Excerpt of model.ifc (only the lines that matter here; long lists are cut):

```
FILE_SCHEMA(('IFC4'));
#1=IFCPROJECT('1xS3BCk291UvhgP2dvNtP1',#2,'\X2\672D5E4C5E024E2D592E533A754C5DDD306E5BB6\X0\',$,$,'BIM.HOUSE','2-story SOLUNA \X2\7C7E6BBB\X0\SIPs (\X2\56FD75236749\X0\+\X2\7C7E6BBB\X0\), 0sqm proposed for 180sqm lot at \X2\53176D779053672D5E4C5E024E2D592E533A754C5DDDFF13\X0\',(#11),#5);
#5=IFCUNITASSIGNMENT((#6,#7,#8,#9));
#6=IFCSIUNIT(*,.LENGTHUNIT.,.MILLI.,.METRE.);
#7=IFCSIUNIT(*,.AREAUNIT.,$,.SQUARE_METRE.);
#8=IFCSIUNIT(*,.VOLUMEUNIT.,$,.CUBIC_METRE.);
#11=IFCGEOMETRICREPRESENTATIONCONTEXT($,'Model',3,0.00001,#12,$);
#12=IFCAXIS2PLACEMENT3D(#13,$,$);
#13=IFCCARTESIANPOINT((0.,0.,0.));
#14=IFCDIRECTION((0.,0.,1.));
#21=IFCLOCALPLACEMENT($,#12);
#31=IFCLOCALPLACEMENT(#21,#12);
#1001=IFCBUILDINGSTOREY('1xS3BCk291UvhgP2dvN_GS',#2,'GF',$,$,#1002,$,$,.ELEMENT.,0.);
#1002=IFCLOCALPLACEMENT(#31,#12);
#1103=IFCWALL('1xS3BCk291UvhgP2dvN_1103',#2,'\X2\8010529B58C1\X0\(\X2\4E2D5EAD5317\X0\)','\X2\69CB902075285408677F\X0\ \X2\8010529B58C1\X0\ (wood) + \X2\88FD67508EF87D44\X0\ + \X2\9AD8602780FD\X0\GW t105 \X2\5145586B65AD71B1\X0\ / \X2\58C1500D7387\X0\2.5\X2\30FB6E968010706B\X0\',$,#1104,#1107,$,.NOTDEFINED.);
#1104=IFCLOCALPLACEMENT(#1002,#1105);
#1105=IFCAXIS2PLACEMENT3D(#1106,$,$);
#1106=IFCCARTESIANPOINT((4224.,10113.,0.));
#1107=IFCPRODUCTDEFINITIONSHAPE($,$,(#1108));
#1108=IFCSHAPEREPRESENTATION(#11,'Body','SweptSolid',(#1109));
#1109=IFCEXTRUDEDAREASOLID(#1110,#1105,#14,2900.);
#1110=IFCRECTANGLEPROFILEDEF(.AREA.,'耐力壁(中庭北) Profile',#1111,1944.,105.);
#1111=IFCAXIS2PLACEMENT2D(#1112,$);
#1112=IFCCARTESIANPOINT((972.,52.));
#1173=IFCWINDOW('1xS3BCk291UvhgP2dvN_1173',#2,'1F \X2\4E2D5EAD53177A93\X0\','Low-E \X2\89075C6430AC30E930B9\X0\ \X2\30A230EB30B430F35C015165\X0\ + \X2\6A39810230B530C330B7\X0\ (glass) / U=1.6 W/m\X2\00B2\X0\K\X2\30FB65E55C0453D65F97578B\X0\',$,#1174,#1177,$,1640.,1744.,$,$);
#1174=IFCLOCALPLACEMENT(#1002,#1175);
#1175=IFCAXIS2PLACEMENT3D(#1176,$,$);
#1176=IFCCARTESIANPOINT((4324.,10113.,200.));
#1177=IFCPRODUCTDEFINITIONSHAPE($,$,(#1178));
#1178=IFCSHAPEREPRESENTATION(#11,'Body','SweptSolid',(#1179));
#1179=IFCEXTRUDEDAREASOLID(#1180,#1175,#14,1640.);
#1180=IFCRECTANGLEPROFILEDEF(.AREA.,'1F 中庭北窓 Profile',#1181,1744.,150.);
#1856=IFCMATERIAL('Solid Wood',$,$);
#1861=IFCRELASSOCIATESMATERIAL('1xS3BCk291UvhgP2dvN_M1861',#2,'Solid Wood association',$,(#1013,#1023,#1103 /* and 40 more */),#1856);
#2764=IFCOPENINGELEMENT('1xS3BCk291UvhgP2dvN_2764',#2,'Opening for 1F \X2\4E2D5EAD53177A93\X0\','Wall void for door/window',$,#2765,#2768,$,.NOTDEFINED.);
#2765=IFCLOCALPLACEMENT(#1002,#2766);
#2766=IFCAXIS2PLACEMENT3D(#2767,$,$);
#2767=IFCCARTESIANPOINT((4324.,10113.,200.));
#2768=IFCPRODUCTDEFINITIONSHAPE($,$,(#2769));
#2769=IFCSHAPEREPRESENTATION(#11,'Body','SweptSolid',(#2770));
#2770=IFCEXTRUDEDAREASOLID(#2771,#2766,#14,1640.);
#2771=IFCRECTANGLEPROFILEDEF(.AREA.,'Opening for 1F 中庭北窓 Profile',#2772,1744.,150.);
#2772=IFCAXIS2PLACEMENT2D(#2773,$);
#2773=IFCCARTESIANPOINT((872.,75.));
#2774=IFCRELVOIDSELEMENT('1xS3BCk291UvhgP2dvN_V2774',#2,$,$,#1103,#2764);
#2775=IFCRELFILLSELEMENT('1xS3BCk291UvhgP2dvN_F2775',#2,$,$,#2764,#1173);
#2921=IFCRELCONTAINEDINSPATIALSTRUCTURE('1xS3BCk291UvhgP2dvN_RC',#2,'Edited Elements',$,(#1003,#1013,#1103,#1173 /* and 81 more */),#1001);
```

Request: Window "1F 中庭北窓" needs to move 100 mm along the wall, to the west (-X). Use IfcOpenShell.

```python
import ifcopenshell
import ifcopenshell.api.geometry
import ifcopenshell.util.placement

model = ifcopenshell.open("model.ifc")

window = model.by_id(1173)
opening = window.FillsVoids[0].RelatingOpeningElement
wall = opening.VoidsElements[0].RelatingBuildingElement

wall_matrix = ifcopenshell.util.placement.get_local_placement(wall.ObjectPlacement)
shift = wall_matrix[:3, 0] * -100.0
before = ifcopenshell.util.placement.get_local_placement(window.ObjectPlacement)[:3, 3].copy()

# The window is not placed relative to its opening, so move both.
for product in (opening, window):
    matrix = ifcopenshell.util.placement.get_local_placement(product.ObjectPlacement)
    matrix[:3, 3] += shift
    ifcopenshell.api.geometry.edit_object_placement(model, product=product, matrix=matrix, is_si=False)

after = ifcopenshell.util.placement.get_local_placement(window.ObjectPlacement)[:3, 3]
print("window moved by", (after - before).round(3) + 0.0)

model.write("model_updated.ifc")
```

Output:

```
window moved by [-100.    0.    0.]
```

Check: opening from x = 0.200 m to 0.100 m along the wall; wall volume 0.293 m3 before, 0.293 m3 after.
